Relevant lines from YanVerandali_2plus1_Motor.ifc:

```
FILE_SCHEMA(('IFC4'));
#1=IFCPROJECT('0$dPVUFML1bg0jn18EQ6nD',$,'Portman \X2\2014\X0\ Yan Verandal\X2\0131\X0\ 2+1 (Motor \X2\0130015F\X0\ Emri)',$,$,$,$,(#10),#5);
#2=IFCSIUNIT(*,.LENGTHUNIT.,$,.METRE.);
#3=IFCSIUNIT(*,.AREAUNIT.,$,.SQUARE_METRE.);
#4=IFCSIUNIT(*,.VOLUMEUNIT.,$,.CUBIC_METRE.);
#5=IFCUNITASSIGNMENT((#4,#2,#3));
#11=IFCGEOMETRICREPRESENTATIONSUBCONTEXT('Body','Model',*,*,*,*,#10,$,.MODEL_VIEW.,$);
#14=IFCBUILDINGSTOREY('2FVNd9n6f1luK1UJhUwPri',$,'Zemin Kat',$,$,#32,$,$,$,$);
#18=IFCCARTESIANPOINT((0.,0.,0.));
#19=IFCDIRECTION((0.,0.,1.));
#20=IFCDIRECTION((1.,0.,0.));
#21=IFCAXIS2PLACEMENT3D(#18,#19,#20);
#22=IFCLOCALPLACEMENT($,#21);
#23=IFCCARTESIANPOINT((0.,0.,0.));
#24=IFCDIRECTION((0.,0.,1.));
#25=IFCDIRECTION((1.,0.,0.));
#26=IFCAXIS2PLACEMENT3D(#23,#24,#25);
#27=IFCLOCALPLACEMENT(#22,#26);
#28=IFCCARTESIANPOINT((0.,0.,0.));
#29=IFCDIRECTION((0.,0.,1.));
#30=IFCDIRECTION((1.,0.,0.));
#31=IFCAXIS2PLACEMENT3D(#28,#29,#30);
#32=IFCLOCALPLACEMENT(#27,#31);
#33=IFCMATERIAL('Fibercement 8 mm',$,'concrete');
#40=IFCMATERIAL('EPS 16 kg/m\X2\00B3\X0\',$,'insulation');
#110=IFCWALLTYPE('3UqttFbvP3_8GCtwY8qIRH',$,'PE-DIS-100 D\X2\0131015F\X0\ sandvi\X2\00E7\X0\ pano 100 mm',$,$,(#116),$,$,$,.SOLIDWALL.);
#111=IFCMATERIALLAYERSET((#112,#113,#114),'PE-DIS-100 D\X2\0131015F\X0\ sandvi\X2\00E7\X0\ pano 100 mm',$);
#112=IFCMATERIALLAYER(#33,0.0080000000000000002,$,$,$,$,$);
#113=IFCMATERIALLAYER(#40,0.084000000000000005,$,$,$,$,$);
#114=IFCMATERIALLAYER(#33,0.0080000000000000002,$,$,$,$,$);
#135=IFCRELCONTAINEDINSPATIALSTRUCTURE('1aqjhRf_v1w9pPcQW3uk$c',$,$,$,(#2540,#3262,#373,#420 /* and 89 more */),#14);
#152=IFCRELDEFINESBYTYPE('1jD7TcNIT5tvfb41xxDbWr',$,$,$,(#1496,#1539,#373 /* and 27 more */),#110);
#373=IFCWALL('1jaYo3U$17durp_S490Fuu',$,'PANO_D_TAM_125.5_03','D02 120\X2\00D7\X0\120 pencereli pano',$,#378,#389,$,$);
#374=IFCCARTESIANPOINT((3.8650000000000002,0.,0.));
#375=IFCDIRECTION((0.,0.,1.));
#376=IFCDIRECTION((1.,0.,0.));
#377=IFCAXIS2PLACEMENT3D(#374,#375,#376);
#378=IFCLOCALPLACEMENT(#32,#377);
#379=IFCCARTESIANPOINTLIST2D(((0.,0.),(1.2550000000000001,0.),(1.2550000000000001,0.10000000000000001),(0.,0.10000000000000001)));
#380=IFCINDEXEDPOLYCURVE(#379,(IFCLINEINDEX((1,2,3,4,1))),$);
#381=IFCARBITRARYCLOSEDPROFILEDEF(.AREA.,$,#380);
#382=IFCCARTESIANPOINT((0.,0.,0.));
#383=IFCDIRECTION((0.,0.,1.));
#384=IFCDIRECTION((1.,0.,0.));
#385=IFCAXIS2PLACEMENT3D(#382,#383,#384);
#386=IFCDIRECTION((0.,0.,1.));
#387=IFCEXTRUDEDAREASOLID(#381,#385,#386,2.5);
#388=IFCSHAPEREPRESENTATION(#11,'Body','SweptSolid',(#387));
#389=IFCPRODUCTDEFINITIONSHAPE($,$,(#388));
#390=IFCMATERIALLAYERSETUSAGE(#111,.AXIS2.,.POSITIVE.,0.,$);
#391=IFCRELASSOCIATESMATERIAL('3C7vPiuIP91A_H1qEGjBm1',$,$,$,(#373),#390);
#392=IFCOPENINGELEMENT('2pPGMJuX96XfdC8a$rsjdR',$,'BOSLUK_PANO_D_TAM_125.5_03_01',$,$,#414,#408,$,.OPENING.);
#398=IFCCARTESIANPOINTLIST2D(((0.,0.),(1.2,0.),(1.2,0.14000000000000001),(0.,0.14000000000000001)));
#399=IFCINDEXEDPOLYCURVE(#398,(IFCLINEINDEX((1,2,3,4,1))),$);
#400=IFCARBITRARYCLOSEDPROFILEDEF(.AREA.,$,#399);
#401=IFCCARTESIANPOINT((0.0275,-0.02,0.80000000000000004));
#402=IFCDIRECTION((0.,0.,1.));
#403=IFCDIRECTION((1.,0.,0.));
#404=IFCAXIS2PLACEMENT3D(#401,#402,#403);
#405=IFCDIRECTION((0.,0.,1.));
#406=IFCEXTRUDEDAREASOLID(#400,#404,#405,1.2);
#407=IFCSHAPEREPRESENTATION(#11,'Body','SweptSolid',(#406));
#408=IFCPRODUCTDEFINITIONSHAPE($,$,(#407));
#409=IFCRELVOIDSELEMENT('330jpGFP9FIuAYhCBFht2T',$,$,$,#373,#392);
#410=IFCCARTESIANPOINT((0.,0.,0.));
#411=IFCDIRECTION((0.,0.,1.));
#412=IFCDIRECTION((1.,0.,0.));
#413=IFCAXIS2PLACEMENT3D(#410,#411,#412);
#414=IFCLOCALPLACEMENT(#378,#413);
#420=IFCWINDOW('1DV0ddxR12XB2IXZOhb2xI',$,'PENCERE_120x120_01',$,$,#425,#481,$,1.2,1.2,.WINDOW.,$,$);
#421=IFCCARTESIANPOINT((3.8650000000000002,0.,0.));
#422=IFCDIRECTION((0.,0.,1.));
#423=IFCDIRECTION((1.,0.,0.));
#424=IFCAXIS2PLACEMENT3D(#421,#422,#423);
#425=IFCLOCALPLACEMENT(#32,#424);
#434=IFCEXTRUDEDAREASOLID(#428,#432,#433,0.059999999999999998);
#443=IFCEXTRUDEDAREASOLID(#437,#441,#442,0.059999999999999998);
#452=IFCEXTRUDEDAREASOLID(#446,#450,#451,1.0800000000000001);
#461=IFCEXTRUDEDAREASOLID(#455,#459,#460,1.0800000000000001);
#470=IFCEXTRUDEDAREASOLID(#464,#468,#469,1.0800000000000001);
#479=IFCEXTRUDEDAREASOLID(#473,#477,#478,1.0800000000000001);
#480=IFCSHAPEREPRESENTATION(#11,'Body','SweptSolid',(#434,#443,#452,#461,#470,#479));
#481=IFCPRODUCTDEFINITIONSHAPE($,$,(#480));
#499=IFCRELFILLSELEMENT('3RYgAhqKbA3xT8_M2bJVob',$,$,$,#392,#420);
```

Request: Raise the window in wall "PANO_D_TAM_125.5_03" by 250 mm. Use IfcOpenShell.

```python
import numpy as np
import ifcopenshell
import ifcopenshell.api.geometry
import ifcopenshell.util.placement
import ifcopenshell.util.unit

model = ifcopenshell.open("YanVerandali_2plus1_Motor.ifc")
unit_scale = ifcopenshell.util.unit.calculate_unit_scale(model)

window = model.by_guid("1DV0ddxR12XB2IXZOhb2xI")
opening = window.FillsVoids[0].RelatingOpeningElement
dz = 0.25

shift = np.array([0.0, 0.0, dz])
# The window is not placed relative to its opening, so move both.
for product in (opening, window):
    matrix = ifcopenshell.util.placement.get_local_placement(product.ObjectPlacement)
    matrix[:3, 3] += shift
    ifcopenshell.api.geometry.edit_object_placement(model, product=product, matrix=matrix, is_si=False)

print(f"moved by {dz * unit_scale:+.3f} m")

model.write("YanVerandali_2plus1_Motor_rev.ifc")
```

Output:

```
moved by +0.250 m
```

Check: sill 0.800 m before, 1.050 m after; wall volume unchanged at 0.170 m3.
